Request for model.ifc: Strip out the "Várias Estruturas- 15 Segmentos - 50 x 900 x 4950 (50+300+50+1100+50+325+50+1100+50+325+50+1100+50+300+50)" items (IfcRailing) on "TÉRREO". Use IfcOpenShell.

First a look at what the model holds.

```python
import ifcopenshell
import ifcopenshell.util.element

model = ifcopenshell.open("model.ifc")
print(model.schema)
storey = next(s for s in model.by_type("IfcBuildingStorey") if s.Name == "TÉRREO")
railings = [e for e in ifcopenshell.util.element.get_decomposition(storey) if e.is_a("IfcRailing")]
seen = {}
for e in railings:
    element_type = ifcopenshell.util.element.get_type(e)
    name = element_type.Name if element_type not in (None, e) else None
    seen[name] = seen.get(name, 0) + 1
for name, count in sorted(seen.items(), key=str):
    print(count, "x", name)
```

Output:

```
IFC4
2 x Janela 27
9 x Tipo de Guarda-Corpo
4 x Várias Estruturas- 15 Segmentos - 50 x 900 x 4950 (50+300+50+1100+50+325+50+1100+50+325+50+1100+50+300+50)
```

```python
import ifcopenshell
import ifcopenshell.api.root
import ifcopenshell.util.element

model = ifcopenshell.open("model.ifc")

storey = next(s for s in model.by_type("IfcBuildingStorey") if s.Name == "TÉRREO")
railings = [e for e in ifcopenshell.util.element.get_decomposition(storey) if e.is_a("IfcRailing")]
targets = [e for e in railings if (t := ifcopenshell.util.element.get_type(e)) not in (None, e) and t.Name == "Várias Estruturas- 15 Segmentos - 50 x 900 x 4950 (50+300+50+1100+50+325+50+1100+50+325+50+1100+50+300+50)"]

for e in targets:
    ifcopenshell.api.root.remove_product(model, product=e)
print(len(targets), "removed")

model.write("model_edited.ifc")
```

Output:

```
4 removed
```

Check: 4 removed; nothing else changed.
